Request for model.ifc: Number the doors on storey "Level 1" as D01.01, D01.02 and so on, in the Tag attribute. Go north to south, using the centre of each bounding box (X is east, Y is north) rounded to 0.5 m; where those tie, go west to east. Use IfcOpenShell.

First a look at what the model holds.

```python
import ifcopenshell
import ifcopenshell.util.element
import ifcopenshell.util.placement

model = ifcopenshell.open("model.ifc")
print(model.schema)
storey = next(s for s in model.by_type("IfcBuildingStorey") if s.Name == "Level 1")
doors = [e for e in ifcopenshell.util.element.get_decomposition(storey) if e.is_a("IfcDoor")]
for e in sorted(doors, key=lambda e: e.id()):
    origin = ifcopenshell.util.placement.get_local_placement(e.ObjectPlacement)[:3, 3]
    print(e.id(), e.Tag, e.Name, origin.round(2) + 0.0, sep=" | ")
```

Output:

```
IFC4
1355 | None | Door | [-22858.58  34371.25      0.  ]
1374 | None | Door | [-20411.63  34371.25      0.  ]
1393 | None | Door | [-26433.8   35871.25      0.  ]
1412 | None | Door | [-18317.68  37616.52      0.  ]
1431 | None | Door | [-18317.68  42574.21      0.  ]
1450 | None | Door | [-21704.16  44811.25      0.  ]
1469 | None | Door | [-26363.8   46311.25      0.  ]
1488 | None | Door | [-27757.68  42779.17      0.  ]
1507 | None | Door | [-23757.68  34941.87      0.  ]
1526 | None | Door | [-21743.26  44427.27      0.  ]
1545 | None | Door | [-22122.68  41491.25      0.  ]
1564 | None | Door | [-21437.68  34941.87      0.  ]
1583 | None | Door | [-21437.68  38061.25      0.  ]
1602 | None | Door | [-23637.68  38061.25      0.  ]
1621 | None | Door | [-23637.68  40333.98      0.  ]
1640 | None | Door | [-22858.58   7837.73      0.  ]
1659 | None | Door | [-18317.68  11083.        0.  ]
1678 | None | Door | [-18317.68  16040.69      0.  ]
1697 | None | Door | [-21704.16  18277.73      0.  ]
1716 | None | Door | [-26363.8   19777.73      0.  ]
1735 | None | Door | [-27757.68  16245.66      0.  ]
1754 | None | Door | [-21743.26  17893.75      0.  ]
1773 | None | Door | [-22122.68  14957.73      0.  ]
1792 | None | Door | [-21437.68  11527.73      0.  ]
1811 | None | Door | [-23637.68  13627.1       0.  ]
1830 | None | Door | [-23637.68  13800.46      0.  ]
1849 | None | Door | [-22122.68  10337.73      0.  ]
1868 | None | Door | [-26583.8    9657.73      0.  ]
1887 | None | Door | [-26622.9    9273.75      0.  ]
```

```python
import ifcopenshell
import ifcopenshell.geom
import ifcopenshell.util.element
import ifcopenshell.util.shape

model = ifcopenshell.open("model.ifc")
settings = ifcopenshell.geom.settings()
settings.set("use-world-coords", True)


def centre(element):
    shape = ifcopenshell.geom.create_shape(settings, element)
    return ifcopenshell.util.shape.get_bbox_centroid(shape.geometry)


storey = next(s for s in model.by_type("IfcBuildingStorey") if s.Name == "Level 1")
doors = [e for e in ifcopenshell.util.element.get_decomposition(storey) if e.is_a("IfcDoor")]

# Insertion points can sit at a corner or the storey origin, so sort by the geometry (in metres).
centres = {e: centre(e) for e in doors}
doors.sort(key=lambda e: (-round(centres[e][1] / 0.5), centres[e][0]))

for i, e in enumerate(doors, start=1):
    number = f"D01.{i:02d}"
    e.Tag = number
    print(e.id(), number)

model.write("model_edited.ifc")
```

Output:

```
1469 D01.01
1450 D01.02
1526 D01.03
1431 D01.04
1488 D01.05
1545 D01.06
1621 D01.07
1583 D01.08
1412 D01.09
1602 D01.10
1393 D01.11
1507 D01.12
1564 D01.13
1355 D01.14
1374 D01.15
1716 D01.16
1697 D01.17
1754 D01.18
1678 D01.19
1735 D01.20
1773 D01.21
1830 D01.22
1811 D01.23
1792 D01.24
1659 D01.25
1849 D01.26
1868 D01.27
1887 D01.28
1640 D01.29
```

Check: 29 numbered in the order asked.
